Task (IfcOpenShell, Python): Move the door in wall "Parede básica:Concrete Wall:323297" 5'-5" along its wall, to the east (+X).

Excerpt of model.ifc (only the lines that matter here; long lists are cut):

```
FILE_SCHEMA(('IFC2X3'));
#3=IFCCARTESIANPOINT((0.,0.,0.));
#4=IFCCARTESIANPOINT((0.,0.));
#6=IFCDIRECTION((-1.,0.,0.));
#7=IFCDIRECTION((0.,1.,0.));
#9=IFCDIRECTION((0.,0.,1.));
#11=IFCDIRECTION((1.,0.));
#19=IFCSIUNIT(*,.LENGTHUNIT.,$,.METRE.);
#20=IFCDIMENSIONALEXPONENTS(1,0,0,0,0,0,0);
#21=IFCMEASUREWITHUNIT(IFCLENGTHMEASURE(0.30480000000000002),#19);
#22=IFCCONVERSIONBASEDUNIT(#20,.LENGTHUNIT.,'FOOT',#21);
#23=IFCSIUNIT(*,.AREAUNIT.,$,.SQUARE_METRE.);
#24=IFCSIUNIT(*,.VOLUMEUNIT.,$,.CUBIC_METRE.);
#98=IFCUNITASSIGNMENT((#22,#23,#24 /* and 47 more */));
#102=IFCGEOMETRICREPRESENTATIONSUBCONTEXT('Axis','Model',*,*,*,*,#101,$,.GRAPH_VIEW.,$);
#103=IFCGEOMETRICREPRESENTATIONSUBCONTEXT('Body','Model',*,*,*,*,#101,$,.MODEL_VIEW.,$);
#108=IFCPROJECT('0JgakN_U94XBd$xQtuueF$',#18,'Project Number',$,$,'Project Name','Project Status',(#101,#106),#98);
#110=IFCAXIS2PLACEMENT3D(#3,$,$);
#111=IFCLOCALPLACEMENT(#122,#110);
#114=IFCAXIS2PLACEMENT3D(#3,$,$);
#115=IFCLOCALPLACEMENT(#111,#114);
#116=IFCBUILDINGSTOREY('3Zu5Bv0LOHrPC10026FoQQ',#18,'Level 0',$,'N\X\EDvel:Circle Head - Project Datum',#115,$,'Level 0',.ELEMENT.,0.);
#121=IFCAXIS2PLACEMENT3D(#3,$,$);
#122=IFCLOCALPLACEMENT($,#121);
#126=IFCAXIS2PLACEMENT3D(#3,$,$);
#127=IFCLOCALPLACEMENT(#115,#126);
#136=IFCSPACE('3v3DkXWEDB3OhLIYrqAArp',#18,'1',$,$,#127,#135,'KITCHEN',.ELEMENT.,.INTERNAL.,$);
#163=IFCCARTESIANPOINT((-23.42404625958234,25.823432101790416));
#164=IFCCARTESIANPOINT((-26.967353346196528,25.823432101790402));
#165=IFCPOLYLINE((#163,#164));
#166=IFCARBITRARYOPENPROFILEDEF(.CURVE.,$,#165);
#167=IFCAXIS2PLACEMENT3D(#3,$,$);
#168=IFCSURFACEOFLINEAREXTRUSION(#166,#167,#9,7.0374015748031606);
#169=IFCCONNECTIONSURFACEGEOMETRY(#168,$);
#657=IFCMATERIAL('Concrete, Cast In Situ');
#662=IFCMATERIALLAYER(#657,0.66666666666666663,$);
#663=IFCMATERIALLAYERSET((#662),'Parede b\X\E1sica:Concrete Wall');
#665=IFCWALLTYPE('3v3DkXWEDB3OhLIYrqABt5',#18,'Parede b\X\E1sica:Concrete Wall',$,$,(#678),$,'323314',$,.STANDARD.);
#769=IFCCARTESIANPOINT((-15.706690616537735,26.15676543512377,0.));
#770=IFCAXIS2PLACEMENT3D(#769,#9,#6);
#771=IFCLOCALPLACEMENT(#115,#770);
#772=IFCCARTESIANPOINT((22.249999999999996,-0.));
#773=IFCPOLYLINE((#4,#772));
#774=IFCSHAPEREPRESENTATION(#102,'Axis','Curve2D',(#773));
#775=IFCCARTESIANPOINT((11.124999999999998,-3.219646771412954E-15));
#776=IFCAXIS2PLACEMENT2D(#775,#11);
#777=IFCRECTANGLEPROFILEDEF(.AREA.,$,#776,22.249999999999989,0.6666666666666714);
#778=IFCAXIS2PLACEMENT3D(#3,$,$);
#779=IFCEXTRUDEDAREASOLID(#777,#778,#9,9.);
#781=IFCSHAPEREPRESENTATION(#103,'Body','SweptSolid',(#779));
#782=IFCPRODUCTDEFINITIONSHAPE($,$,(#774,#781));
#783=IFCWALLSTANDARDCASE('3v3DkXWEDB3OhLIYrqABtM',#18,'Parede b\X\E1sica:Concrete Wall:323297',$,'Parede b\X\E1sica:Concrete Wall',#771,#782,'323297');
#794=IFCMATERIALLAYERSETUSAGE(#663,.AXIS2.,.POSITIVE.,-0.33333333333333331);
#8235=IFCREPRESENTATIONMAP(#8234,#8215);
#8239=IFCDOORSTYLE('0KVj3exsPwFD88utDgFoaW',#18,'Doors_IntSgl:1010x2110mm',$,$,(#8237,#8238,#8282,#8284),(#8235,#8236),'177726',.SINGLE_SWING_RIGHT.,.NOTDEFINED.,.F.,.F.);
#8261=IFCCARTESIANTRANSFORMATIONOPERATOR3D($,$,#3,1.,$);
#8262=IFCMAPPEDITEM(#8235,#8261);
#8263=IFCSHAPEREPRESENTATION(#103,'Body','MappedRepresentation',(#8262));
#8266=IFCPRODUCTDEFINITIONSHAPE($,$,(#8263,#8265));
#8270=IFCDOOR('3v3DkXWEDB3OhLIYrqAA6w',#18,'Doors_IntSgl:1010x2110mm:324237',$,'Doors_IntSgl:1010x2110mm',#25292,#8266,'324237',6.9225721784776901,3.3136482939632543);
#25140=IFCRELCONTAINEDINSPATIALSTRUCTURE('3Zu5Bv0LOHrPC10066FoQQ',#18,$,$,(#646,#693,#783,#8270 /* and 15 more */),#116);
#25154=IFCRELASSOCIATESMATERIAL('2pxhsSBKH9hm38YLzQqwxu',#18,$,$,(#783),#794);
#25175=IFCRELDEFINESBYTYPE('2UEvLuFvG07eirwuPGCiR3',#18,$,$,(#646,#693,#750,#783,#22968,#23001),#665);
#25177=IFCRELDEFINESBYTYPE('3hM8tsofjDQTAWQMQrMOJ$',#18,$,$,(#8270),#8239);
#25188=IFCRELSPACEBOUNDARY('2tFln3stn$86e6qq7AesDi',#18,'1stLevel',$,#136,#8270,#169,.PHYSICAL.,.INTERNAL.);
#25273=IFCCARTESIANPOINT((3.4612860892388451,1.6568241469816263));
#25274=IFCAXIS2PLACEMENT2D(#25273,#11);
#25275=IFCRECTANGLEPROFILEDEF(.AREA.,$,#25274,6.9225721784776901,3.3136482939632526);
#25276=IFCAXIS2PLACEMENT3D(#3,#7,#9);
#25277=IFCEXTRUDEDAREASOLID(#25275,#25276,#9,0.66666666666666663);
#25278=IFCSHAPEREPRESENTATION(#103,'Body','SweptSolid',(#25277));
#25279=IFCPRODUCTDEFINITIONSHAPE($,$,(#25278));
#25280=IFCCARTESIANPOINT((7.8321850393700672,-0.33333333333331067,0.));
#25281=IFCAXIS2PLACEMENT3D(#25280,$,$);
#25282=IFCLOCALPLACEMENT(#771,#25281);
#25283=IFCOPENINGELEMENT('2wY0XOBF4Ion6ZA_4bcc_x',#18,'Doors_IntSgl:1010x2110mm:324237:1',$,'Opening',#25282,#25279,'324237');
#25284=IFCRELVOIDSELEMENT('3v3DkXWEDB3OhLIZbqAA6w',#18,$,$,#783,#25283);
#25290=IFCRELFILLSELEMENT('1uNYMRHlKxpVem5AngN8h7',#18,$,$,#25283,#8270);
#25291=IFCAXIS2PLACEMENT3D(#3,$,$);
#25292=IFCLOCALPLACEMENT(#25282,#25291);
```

```python
import numpy as np
import ifcopenshell
import ifcopenshell.api.geometry
import ifcopenshell.util.placement
import ifcopenshell.util.unit

model = ifcopenshell.open("model.ifc")
unit_scale = ifcopenshell.util.unit.calculate_unit_scale(model)

door = model.by_guid("3v3DkXWEDB3OhLIYrqAA6w")
opening = door.FillsVoids[0].RelatingOpeningElement
wall = opening.VoidsElements[0].RelatingBuildingElement

wall_matrix = ifcopenshell.util.placement.get_local_placement(wall.ObjectPlacement)
shift = wall_matrix[:3, 0] * -65 * 0.0254 / unit_scale
before = ifcopenshell.util.placement.get_local_placement(door.ObjectPlacement)[:3, 3].copy()

# The door is placed relative to its opening, so it follows when the opening moves.
matrix = ifcopenshell.util.placement.get_local_placement(opening.ObjectPlacement)
matrix[:3, 3] += shift
ifcopenshell.api.geometry.edit_object_placement(
    model, product=opening, matrix=matrix, is_si=False, should_transform_children=True
)

# Space boundary surfaces are stored in each space's coordinates; move them too.
for rel in door.ProvidesBoundaries:
    if not rel.ConnectionGeometry:
        continue
    surface = rel.ConnectionGeometry.SurfaceOnRelatingElement
    space_matrix = ifcopenshell.util.placement.get_local_placement(rel.RelatingSpace.ObjectPlacement)
    point = np.array(surface.Position.Location.Coordinates) + space_matrix[:3, :3].T @ shift
    surface.Position = model.createIfcAxis2Placement3D(
        model.createIfcCartesianPoint(point.tolist()), surface.Position.Axis, surface.Position.RefDirection
    )

after = ifcopenshell.util.placement.get_local_placement(door.ObjectPlacement)[:3, 3]
print("door moved by", (after - before).round(3) + 0.0)

model.write("model_rev.ifc")
```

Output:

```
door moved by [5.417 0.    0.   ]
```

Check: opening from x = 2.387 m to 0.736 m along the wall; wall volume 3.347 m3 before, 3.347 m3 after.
